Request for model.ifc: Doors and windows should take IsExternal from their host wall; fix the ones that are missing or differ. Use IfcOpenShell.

First a look at what the model holds.

```python
import ifcopenshell
import ifcopenshell.util.element

model = ifcopenshell.open("model.ifc")
print(model.schema)
seen = {}
for e in model.by_type("IfcDoor") + model.by_type("IfcWindow"):
    if not e.FillsVoids:
        continue
    host = e.FillsVoids[0].RelatingOpeningElement.VoidsElements[0].RelatingBuildingElement
    own = ifcopenshell.util.element.get_pset(e, f"Pset_{e.is_a()[3:].removesuffix('StandardCase')}Common", "IsExternal")
    wall = ifcopenshell.util.element.get_pset(host, "Pset_WallCommon", "IsExternal")
    seen[e.is_a(), own, wall] = seen.get((e.is_a(), own, wall), 0) + 1
for (cls, own, wall), count in sorted(seen.items(), key=str):
    print(count, cls, "IsExternal:", own, "| host wall:", wall)
```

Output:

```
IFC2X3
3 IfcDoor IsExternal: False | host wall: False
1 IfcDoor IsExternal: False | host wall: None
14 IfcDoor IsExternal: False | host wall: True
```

```python
import ifcopenshell
import ifcopenshell.api.pset
import ifcopenshell.util.element

model = ifcopenshell.open("model.ifc")

count = 0
for ifc_class, pset_name in (("IfcDoor", "Pset_DoorCommon"), ("IfcWindow", "Pset_WindowCommon")):
    for e in model.by_type(ifc_class):
        if not e.FillsVoids:
            continue
        host = e.FillsVoids[0].RelatingOpeningElement.VoidsElements[0].RelatingBuildingElement
        external = ifcopenshell.util.element.get_pset(host, "Pset_WallCommon", "IsExternal")
        if external is None or ifcopenshell.util.element.get_pset(e, pset_name, "IsExternal") == external:
            continue
        pset = ifcopenshell.api.pset.add_pset(model, product=e, name=pset_name)
        ifcopenshell.api.pset.edit_pset(model, pset=pset, properties={"IsExternal": external})
        count += 1

print(count, "updated")

model.write("model_edited.ifc")
```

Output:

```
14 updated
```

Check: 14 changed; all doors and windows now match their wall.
